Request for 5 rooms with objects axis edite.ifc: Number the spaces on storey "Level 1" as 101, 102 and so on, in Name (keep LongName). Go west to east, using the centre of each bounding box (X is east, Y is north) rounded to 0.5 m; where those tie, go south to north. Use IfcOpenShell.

First a look at what the model holds.

```python
import ifcopenshell
import ifcopenshell.util.element
import ifcopenshell.util.placement

model = ifcopenshell.open("5 rooms with objects axis edite.ifc")
print(model.schema)
storey = next(s for s in model.by_type("IfcBuildingStorey") if s.Name == "Level 1")
spaces = [e for e in ifcopenshell.util.element.get_decomposition(storey) if e.is_a("IfcSpace")]
for e in sorted(spaces, key=lambda e: e.id()):
    origin = ifcopenshell.util.placement.get_local_placement(e.ObjectPlacement)[:3, 3]
    print(e.id(), e.Name, e.LongName, origin.round(2) + 0.0, sep=" | ")
```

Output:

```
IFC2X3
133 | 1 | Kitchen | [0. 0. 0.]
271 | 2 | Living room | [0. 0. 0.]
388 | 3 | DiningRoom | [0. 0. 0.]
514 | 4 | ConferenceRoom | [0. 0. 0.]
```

```python
import ifcopenshell
import ifcopenshell.geom
import ifcopenshell.util.element
import ifcopenshell.util.shape

model = ifcopenshell.open("5 rooms with objects axis edite.ifc")
settings = ifcopenshell.geom.settings()
settings.set("use-world-coords", True)


def centre(element):
    shape = ifcopenshell.geom.create_shape(settings, element)
    return ifcopenshell.util.shape.get_bbox_centroid(shape.geometry)


storey = next(s for s in model.by_type("IfcBuildingStorey") if s.Name == "Level 1")
spaces = [e for e in ifcopenshell.util.element.get_decomposition(storey) if e.is_a("IfcSpace")]

# Insertion points can sit at a corner or the storey origin, so sort by the geometry (in metres).
centres = {e: centre(e) for e in spaces}
spaces.sort(key=lambda e: (round(centres[e][0] / 0.5), centres[e][1]))

for i, e in enumerate(spaces, start=1):
    number = f"1{i:02d}"
    e.Name = number
    print(e.id(), number)

model.write("5 rooms with objects axis edite_v2.ifc")
```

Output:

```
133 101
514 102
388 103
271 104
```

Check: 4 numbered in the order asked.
